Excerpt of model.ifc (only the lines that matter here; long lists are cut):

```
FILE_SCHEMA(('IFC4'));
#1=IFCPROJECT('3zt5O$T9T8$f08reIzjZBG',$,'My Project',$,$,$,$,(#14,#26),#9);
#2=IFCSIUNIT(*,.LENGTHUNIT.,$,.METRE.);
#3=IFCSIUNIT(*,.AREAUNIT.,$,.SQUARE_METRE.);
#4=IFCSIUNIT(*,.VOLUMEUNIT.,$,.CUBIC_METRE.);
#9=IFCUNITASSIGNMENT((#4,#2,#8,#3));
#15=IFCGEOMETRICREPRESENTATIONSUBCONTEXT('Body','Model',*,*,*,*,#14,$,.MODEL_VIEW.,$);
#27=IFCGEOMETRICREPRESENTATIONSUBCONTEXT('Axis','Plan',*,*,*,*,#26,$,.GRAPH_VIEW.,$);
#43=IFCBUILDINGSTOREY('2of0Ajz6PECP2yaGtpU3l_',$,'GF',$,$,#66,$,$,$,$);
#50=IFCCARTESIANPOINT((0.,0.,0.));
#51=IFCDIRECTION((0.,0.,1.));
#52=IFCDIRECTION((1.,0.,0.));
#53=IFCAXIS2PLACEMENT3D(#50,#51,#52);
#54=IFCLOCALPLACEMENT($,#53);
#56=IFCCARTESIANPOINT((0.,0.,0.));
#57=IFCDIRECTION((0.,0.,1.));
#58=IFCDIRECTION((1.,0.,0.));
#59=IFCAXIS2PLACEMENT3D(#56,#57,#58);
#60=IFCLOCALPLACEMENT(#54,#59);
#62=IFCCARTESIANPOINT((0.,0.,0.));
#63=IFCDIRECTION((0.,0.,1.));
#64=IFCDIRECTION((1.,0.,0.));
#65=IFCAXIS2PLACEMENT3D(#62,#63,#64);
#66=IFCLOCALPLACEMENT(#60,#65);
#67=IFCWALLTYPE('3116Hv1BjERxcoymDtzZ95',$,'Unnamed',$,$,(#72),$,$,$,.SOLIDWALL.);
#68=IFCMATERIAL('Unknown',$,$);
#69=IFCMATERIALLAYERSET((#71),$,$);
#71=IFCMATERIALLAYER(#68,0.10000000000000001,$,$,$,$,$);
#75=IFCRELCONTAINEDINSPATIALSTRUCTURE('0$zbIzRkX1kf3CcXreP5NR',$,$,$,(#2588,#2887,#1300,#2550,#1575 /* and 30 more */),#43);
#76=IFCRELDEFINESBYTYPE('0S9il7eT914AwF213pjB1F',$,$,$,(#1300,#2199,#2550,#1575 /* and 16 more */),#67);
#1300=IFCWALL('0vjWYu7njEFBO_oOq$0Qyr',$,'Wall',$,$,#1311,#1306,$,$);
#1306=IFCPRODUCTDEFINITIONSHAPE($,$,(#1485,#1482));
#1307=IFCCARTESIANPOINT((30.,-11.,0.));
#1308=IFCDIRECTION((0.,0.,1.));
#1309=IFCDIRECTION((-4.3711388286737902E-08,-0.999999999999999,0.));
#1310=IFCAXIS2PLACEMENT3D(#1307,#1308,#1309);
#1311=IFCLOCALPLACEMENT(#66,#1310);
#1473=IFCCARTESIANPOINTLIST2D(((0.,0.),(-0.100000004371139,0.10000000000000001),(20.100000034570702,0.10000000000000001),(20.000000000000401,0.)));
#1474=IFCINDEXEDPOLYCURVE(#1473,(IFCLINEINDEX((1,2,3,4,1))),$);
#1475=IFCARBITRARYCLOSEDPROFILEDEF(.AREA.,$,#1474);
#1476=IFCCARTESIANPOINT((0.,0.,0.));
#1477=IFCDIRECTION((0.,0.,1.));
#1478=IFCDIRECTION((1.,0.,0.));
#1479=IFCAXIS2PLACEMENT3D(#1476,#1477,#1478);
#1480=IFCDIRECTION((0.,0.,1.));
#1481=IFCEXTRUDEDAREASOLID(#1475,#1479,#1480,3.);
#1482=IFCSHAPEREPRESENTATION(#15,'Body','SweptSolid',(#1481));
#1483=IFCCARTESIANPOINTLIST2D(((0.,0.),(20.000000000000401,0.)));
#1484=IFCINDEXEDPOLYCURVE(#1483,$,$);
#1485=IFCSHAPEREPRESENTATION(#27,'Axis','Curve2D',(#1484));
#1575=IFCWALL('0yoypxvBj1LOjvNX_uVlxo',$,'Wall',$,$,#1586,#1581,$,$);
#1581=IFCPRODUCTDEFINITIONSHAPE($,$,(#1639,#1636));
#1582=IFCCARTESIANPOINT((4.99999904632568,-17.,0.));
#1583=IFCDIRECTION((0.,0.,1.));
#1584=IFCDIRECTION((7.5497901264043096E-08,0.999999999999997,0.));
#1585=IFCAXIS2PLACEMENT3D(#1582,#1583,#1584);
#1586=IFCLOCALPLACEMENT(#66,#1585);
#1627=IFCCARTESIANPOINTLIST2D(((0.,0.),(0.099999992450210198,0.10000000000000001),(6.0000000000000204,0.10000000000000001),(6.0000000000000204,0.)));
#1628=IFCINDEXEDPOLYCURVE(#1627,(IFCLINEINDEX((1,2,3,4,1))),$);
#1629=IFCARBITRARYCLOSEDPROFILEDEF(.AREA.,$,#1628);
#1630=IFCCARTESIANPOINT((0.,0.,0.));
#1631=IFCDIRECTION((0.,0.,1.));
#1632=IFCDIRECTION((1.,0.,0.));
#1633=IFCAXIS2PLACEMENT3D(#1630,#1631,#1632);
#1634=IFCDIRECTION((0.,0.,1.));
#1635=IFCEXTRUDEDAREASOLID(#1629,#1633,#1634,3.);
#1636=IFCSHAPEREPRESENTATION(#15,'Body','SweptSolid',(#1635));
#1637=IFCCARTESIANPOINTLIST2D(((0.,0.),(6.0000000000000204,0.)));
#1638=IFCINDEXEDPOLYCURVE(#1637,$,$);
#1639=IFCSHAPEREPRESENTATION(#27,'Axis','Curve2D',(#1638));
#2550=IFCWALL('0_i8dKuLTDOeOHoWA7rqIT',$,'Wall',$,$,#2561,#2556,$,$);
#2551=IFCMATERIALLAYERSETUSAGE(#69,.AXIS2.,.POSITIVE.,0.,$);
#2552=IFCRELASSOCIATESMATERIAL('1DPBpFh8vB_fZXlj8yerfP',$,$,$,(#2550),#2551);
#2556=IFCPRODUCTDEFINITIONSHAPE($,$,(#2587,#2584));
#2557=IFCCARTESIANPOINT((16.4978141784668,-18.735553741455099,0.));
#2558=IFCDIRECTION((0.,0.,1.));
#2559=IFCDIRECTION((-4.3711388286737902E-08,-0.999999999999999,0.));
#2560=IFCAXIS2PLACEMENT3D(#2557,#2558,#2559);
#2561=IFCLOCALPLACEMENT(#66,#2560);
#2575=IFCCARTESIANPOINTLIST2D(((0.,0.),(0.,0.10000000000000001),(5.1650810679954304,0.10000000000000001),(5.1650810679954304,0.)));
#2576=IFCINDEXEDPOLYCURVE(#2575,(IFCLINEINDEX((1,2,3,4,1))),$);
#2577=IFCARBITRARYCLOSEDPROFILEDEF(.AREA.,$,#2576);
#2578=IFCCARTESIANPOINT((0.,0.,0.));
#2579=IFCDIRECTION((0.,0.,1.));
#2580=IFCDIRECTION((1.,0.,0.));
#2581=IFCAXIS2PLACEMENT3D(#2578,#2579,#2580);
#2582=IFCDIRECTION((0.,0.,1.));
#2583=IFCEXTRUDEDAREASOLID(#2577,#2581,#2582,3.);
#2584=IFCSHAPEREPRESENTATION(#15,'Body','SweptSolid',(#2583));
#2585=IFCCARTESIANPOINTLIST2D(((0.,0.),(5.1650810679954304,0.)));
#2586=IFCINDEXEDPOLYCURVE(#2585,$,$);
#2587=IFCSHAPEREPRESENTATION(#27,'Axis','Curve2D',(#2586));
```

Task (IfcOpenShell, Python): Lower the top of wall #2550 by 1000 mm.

```python
import ifcopenshell
import ifcopenshell.geom
import ifcopenshell.util.representation
import ifcopenshell.util.shape

model = ifcopenshell.open("model.ifc")
settings = ifcopenshell.geom.settings()


def volume(element):
    """Net volume in cubic metres, openings subtracted."""
    shape = ifcopenshell.geom.create_shape(settings, element)
    return ifcopenshell.util.shape.get_volume(shape.geometry)


wall = model.by_guid("0_i8dKuLTDOeOHoWA7rqIT")
before = volume(wall)

body = ifcopenshell.util.representation.get_representation(wall, "Model", "Body")
solid = body.Items[0]
old_height = solid.Depth
solid.Depth -= 1.0
after = volume(wall)

print(f"height {old_height:g} -> {solid.Depth:g}, volume {before:.3f} -> {after:.3f} m3")

model.write("model_updated.ifc")
```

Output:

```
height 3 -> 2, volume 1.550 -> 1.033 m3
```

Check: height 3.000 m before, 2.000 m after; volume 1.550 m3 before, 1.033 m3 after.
